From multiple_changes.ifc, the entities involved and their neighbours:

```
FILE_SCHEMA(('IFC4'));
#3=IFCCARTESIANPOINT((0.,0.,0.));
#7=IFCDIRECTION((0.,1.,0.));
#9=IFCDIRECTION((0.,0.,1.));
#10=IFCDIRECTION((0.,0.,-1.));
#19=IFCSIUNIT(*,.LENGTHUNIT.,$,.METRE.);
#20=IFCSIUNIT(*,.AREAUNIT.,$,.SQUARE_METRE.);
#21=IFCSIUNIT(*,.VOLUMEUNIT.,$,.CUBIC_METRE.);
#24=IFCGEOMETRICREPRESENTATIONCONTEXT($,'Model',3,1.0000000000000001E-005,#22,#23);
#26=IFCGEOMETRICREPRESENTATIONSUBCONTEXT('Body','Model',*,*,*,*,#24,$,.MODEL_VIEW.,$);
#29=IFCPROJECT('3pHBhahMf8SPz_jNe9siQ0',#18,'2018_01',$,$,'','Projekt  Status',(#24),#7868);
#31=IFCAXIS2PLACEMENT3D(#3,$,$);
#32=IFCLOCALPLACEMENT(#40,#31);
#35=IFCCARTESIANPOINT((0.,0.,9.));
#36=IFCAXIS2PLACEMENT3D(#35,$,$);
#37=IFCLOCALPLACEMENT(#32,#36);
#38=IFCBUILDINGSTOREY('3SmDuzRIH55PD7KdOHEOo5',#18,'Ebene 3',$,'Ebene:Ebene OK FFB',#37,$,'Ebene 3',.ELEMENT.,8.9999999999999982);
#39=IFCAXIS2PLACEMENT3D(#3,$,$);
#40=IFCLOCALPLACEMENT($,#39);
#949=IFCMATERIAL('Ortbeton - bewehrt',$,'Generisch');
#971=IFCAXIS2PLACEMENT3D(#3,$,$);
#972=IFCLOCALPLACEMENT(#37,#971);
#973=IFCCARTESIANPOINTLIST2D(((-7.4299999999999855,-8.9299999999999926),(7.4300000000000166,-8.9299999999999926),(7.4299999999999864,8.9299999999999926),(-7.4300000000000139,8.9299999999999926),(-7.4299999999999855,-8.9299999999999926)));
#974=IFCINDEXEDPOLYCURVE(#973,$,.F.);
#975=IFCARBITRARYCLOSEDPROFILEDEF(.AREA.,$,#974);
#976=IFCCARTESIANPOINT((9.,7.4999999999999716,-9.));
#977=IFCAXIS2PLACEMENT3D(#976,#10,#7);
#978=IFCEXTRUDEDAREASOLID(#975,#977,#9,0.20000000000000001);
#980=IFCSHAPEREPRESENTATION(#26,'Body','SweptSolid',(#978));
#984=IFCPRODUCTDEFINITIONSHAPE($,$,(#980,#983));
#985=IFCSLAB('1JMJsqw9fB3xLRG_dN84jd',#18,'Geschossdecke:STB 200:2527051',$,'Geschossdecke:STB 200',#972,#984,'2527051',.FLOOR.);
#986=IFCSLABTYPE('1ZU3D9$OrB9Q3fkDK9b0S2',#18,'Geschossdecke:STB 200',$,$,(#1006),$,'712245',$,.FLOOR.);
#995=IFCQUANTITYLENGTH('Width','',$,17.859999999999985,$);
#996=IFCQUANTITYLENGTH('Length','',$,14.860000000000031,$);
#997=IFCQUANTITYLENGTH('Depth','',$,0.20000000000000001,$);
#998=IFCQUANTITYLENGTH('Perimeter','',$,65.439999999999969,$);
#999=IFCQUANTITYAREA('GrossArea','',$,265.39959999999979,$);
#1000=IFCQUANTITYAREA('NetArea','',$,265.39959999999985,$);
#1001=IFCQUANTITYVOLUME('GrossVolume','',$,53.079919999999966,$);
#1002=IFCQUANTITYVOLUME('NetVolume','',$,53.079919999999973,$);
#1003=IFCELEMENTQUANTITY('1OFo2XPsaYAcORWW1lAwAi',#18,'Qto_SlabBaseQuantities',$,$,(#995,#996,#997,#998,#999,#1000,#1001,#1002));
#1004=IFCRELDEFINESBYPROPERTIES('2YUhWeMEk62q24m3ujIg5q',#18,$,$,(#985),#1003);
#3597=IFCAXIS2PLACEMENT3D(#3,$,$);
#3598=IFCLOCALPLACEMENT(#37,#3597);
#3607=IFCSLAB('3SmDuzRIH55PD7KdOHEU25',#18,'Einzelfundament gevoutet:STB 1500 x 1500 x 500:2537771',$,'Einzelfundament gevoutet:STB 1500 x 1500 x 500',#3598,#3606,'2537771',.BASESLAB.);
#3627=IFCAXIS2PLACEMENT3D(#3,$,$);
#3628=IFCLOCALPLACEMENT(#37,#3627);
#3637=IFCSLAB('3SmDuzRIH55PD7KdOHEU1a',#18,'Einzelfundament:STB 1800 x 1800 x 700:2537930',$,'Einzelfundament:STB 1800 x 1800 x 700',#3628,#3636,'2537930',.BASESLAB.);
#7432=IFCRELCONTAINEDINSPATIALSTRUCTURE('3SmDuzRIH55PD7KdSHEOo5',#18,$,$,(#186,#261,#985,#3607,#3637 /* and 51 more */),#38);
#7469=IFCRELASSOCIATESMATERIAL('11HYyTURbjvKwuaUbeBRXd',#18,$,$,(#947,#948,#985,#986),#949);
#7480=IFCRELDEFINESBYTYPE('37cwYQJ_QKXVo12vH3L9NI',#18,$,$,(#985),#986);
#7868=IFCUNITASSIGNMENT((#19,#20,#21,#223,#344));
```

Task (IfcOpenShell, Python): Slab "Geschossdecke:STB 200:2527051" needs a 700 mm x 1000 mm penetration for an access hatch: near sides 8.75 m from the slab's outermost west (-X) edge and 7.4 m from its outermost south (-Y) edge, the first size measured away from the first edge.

```python
import numpy as np
import ifcopenshell
import ifcopenshell.api.feature
import ifcopenshell.api.geometry
import ifcopenshell.api.pset
import ifcopenshell.api.root
import ifcopenshell.geom
import ifcopenshell.util.element
import ifcopenshell.util.placement
import ifcopenshell.util.representation
import ifcopenshell.util.shape
import ifcopenshell.util.unit

model = ifcopenshell.open("multiple_changes.ifc")
unit_scale = ifcopenshell.util.unit.calculate_unit_scale(model)
area_scale = ifcopenshell.util.unit.calculate_unit_scale(model, "AREAUNIT")
volume_scale = ifcopenshell.util.unit.calculate_unit_scale(model, "VOLUMEUNIT")
settings = ifcopenshell.geom.settings()


def volume(element):
    """Net volume in cubic metres, openings subtracted."""
    shape = ifcopenshell.geom.create_shape(settings, element)
    return ifcopenshell.util.shape.get_volume(shape.geometry)


slab = model.by_id(985)
before = volume(slab)

# Extent in the slab's own axes, in metres. The edges named are its -X and -Y sides.
slab_shape = ifcopenshell.geom.create_shape(settings, slab)
vertices = ifcopenshell.util.shape.get_vertices(slab_shape.geometry)
x_min, y_min, bottom = vertices.min(axis=0)
top = vertices[:, 2].max()

opening = ifcopenshell.api.root.create_entity(model, ifc_class="IfcOpeningElement", name="Access hatch opening", predefined_type="OPENING")
context = ifcopenshell.util.representation.get_context(model, "Model", "Body", "MODEL_VIEW")
width, depth = 0.7, 1
outline = [(0.0, 0.0), (width, 0.0), (width, depth), (0.0, depth), (0.0, 0.0)]
# Overshoot both faces by 50 mm so the cut is clean.
shape = ifcopenshell.api.geometry.add_slab_representation(
    model, context=context, depth=top - bottom + 0.1, polyline=outline
)
ifcopenshell.api.geometry.assign_representation(model, product=opening, representation=shape)

matrix = ifcopenshell.util.placement.get_local_placement(slab.ObjectPlacement)
matrix[:, 3] = matrix @ np.append(np.array([x_min + 8.75, y_min + 7.4, bottom - 0.05]) / unit_scale, 1.0)
ifcopenshell.api.geometry.edit_object_placement(model, product=opening, matrix=matrix, is_si=False)
ifcopenshell.api.feature.add_feature(model, feature=opening, element=slab)

after = volume(slab)

# Update the slab's stored quantities.
qto = model.by_id(ifcopenshell.util.element.get_pset(slab, "Qto_SlabBaseQuantities", should_inherit=False)["id"])
ifcopenshell.api.pset.edit_qto(model, qto=qto, properties={
    "NetArea": after / (top - bottom) / area_scale,
    "NetVolume": after / volume_scale,
})

print(f"slab volume {before:.3f} -> {after:.3f} m3")

model.write("multiple_changes_edited.ifc")
```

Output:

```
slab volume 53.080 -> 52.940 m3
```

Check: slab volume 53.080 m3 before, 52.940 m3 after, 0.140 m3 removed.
